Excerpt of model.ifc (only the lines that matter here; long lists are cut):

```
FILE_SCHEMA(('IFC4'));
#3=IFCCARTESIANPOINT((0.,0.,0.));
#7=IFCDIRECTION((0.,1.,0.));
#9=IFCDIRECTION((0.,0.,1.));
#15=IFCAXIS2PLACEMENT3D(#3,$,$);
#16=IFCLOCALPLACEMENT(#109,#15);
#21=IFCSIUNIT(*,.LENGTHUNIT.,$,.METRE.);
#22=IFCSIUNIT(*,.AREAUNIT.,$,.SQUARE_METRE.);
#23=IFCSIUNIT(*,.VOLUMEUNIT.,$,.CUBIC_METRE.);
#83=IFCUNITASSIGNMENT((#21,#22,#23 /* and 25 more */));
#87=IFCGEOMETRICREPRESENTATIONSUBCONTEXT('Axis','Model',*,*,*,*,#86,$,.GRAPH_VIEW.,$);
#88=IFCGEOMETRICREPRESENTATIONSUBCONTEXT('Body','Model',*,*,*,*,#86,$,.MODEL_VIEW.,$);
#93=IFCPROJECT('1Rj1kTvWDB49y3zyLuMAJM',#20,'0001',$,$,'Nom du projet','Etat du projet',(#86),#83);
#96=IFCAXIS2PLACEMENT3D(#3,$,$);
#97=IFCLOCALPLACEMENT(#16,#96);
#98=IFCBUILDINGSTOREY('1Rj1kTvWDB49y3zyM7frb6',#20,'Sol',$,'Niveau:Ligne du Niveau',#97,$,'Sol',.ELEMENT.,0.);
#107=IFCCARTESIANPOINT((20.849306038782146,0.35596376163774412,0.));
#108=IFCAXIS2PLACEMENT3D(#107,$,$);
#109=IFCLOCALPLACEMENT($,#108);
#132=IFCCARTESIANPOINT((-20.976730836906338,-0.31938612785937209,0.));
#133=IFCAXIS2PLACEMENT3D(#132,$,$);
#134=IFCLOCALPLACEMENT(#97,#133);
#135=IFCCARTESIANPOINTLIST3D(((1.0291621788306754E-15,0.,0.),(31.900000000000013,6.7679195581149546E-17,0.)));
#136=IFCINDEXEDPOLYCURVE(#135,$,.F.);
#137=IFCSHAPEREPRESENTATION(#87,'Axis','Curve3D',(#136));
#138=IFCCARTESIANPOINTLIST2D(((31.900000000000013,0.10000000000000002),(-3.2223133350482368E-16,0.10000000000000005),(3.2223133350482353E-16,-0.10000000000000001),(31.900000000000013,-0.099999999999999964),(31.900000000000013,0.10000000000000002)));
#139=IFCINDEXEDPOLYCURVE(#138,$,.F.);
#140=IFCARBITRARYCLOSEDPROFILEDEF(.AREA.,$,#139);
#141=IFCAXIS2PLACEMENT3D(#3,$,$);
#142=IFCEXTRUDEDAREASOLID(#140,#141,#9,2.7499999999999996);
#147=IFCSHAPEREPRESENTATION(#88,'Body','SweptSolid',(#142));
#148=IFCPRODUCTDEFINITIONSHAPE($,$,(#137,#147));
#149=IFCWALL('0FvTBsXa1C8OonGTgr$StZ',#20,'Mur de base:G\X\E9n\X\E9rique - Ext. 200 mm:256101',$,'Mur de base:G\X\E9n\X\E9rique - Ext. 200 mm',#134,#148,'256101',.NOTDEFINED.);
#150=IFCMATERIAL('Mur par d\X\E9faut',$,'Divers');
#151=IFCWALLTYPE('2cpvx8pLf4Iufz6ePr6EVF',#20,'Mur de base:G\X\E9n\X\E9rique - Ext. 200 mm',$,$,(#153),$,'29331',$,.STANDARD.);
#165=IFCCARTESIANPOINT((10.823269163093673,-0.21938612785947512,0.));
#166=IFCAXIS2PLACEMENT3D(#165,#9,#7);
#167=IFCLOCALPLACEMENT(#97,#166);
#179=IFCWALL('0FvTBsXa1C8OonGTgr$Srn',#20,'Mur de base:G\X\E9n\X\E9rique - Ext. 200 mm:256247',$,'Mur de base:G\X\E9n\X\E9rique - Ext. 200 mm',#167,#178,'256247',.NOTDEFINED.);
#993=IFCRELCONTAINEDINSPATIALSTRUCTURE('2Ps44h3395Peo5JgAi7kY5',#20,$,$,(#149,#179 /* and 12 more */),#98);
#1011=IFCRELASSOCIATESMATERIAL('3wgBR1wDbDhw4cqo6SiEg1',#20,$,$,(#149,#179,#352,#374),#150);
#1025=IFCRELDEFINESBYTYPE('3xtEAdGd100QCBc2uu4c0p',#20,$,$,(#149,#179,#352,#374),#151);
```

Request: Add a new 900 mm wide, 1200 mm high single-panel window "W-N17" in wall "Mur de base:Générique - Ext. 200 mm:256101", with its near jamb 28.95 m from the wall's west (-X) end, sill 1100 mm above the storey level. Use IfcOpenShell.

```python
import numpy as np
import ifcopenshell
import ifcopenshell.api.feature
import ifcopenshell.api.geometry
import ifcopenshell.api.root
import ifcopenshell.api.spatial
import ifcopenshell.geom
import ifcopenshell.util.element
import ifcopenshell.util.placement
import ifcopenshell.util.representation
import ifcopenshell.util.shape
import ifcopenshell.util.unit

model = ifcopenshell.open("model.ifc")
unit_scale = ifcopenshell.util.unit.calculate_unit_scale(model)
settings = ifcopenshell.geom.settings()


def volume(element):
    """Net volume in cubic metres, openings subtracted."""
    shape = ifcopenshell.geom.create_shape(settings, element)
    return ifcopenshell.util.shape.get_volume(shape.geometry)


wall = model.by_id(149)
storey = ifcopenshell.util.element.get_container(wall, ifc_class="IfcBuildingStorey")
context = ifcopenshell.util.representation.get_context(model, "Model", "Body", "MODEL_VIEW")
before = volume(wall)

width, height, from_end, sill = 0.9, 1.2, 28.95, 1.1  # metres

# The wall runs along its own X axis, and the end named is its -X end.
wall_shape = ifcopenshell.geom.create_shape(settings, wall)
x, y, z = ifcopenshell.util.shape.get_vertices(wall_shape.geometry).T
start = x.min() + from_end
face, thickness = float(y.min()), float(y.max() - y.min())
wall_matrix = ifcopenshell.util.placement.get_local_placement(wall.ObjectPlacement)
level = ifcopenshell.util.placement.get_local_placement(storey.ObjectPlacement)[2, 3]


def in_wall(x, y):
    """Placement at x, y metres in the wall's axes, at sill height."""
    matrix = wall_matrix.copy()
    matrix[:, 3] = wall_matrix @ np.array([x / unit_scale, y / unit_scale, 0.0, 1.0])
    matrix[2, 3] = level + sill / unit_scale
    return matrix


# Opening: a box that overshoots both wall faces by 50 mm.
opening = ifcopenshell.api.root.create_entity(model, ifc_class="IfcOpeningElement", predefined_type="OPENING")
box = ifcopenshell.api.geometry.add_wall_representation(
    model, context=context, length=width, height=height, thickness=thickness + 0.1
)
ifcopenshell.api.geometry.assign_representation(model, product=opening, representation=box)
ifcopenshell.api.geometry.edit_object_placement(model, product=opening, matrix=in_wall(start, face - 0.05), is_si=False)
ifcopenshell.api.feature.add_feature(model, feature=opening, element=wall)

window = ifcopenshell.api.root.create_entity(model, ifc_class="IfcWindow", name="W-N17", predefined_type="WINDOW")
window.OverallWidth, window.OverallHeight = width / unit_scale, height / unit_scale
window.PartitioningType = "SINGLE_PANEL"
body = ifcopenshell.api.geometry.add_window_representation(
    model,
    context=context,
    overall_width=window.OverallWidth,
    overall_height=window.OverallHeight,
    partition_type="SINGLE_PANEL",
)
ifcopenshell.api.geometry.assign_representation(model, product=window, representation=body)
ifcopenshell.api.spatial.assign_container(model, products=[window], relating_structure=storey)
ifcopenshell.api.feature.add_filling(model, opening=opening, element=window)

# Centre the window in the wall's thickness.
ifcopenshell.api.geometry.edit_object_placement(model, product=window, matrix=in_wall(start, face), is_si=False)
window_shape = ifcopenshell.geom.create_shape(settings, window)
depth = ifcopenshell.util.shape.get_vertices(window_shape.geometry)[:, 1]
offset = face + thickness / 2 - (depth.min() + depth.max()) / 2
ifcopenshell.api.geometry.edit_object_placement(model, product=window, matrix=in_wall(start, offset), is_si=False)

after = volume(wall)

print(f"wall volume {before:.3f} -> {after:.3f} m3")

model.write("model_v2.ifc")
```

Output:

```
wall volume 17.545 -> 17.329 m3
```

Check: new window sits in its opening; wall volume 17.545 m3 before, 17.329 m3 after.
